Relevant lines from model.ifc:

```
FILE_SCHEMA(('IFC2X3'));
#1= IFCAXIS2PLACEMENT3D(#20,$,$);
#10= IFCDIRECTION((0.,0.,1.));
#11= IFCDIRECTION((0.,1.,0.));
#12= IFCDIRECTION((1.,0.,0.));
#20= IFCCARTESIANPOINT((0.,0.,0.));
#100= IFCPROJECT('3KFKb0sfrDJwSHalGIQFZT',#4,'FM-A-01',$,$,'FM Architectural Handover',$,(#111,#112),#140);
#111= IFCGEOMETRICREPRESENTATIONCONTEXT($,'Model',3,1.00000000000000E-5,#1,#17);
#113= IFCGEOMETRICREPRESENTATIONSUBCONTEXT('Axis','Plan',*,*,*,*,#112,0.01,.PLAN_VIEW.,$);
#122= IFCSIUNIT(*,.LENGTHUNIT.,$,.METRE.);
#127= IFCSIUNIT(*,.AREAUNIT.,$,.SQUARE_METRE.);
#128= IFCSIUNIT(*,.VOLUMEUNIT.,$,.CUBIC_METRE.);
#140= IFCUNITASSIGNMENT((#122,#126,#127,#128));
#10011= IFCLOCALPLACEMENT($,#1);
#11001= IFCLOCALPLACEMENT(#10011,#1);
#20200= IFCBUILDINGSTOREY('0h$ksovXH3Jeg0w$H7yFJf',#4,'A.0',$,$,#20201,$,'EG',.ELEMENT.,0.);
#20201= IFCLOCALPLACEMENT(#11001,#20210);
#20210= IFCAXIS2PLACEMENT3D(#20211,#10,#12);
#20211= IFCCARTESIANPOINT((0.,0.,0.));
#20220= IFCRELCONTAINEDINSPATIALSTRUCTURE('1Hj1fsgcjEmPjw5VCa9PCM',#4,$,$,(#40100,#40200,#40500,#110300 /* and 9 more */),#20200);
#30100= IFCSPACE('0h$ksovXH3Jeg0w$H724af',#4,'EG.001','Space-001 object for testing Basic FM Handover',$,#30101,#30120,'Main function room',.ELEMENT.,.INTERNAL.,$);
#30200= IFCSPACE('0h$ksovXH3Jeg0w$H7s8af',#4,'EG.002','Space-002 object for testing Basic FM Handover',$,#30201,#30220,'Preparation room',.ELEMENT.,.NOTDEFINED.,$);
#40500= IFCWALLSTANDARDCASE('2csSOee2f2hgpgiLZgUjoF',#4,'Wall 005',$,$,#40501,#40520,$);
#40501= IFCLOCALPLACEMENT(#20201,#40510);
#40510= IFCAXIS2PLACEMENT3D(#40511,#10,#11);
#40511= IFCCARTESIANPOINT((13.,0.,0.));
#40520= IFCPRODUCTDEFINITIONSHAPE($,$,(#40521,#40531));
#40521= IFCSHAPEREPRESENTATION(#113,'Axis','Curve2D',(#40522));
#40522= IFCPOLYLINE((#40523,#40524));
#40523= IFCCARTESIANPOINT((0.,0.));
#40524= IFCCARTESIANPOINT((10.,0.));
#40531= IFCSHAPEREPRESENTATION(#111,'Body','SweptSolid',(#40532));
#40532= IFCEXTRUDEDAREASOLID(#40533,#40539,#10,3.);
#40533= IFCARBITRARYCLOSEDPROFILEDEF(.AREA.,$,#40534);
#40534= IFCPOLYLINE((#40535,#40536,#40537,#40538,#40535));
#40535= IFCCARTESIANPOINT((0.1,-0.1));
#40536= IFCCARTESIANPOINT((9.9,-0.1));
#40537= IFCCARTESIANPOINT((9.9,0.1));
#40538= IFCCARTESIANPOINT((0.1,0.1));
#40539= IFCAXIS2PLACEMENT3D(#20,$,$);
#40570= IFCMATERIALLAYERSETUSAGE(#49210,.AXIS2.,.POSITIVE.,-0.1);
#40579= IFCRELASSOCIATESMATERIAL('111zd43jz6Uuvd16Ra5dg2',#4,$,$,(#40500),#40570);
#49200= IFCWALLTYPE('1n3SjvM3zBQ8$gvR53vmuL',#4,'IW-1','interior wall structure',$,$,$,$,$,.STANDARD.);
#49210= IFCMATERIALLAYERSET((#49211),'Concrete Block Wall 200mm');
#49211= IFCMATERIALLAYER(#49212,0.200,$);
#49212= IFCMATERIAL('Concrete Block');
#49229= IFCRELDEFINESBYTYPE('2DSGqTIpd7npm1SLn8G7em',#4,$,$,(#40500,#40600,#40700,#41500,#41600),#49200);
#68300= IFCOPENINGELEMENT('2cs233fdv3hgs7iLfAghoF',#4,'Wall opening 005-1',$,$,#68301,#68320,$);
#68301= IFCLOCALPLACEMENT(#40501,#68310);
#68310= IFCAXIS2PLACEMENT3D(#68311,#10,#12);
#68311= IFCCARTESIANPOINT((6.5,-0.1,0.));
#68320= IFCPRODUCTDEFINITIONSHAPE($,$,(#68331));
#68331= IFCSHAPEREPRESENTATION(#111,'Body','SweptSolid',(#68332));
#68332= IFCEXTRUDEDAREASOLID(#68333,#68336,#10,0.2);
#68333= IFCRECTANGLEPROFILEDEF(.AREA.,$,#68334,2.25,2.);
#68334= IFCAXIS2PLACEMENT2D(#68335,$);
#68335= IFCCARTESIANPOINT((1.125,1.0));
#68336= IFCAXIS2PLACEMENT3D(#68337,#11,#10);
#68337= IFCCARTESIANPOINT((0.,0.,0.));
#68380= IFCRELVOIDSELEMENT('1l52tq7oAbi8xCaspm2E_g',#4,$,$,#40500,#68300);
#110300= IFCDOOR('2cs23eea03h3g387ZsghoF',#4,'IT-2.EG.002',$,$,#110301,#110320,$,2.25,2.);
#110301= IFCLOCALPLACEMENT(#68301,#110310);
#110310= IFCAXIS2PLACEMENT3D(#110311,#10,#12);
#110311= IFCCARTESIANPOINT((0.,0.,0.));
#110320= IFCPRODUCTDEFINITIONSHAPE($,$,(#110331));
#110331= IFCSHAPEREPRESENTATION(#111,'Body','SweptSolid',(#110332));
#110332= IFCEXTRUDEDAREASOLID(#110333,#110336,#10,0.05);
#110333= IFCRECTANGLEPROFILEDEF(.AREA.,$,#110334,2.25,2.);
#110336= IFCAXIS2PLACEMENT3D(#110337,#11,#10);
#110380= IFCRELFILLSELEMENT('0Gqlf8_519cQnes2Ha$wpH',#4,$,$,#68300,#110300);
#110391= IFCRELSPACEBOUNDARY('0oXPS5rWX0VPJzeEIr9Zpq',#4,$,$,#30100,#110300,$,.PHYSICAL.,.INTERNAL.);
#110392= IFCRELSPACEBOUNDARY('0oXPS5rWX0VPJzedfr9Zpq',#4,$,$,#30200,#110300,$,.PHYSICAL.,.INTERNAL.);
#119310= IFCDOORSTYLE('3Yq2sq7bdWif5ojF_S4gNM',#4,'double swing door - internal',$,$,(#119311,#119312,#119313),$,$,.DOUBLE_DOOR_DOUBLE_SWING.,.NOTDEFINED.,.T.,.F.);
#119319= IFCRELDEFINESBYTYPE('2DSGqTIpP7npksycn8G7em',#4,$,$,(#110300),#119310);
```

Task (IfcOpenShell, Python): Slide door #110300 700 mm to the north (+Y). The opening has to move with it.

```python
import ifcopenshell
import ifcopenshell.api.geometry
import ifcopenshell.util.placement
import ifcopenshell.util.unit

model = ifcopenshell.open("model.ifc")
unit_scale = ifcopenshell.util.unit.calculate_unit_scale(model)

door = model.by_guid("2cs23eea03h3g387ZsghoF")
opening = door.FillsVoids[0].RelatingOpeningElement
wall = opening.VoidsElements[0].RelatingBuildingElement

wall_matrix = ifcopenshell.util.placement.get_local_placement(wall.ObjectPlacement)
shift = wall_matrix[:3, 0] * 0.7 / unit_scale
before = ifcopenshell.util.placement.get_local_placement(door.ObjectPlacement)[:3, 3].copy()

# The door is placed relative to its opening, so it follows when the opening moves.
matrix = ifcopenshell.util.placement.get_local_placement(opening.ObjectPlacement)
matrix[:3, 3] += shift
ifcopenshell.api.geometry.edit_object_placement(
    model, product=opening, matrix=matrix, is_si=False, should_transform_children=True
)

after = ifcopenshell.util.placement.get_local_placement(door.ObjectPlacement)[:3, 3]
print("door moved by", (after - before).round(3) + 0.0)

model.write("model_edited.ifc")
```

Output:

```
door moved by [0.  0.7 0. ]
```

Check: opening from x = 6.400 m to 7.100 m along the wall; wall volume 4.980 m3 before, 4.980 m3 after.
